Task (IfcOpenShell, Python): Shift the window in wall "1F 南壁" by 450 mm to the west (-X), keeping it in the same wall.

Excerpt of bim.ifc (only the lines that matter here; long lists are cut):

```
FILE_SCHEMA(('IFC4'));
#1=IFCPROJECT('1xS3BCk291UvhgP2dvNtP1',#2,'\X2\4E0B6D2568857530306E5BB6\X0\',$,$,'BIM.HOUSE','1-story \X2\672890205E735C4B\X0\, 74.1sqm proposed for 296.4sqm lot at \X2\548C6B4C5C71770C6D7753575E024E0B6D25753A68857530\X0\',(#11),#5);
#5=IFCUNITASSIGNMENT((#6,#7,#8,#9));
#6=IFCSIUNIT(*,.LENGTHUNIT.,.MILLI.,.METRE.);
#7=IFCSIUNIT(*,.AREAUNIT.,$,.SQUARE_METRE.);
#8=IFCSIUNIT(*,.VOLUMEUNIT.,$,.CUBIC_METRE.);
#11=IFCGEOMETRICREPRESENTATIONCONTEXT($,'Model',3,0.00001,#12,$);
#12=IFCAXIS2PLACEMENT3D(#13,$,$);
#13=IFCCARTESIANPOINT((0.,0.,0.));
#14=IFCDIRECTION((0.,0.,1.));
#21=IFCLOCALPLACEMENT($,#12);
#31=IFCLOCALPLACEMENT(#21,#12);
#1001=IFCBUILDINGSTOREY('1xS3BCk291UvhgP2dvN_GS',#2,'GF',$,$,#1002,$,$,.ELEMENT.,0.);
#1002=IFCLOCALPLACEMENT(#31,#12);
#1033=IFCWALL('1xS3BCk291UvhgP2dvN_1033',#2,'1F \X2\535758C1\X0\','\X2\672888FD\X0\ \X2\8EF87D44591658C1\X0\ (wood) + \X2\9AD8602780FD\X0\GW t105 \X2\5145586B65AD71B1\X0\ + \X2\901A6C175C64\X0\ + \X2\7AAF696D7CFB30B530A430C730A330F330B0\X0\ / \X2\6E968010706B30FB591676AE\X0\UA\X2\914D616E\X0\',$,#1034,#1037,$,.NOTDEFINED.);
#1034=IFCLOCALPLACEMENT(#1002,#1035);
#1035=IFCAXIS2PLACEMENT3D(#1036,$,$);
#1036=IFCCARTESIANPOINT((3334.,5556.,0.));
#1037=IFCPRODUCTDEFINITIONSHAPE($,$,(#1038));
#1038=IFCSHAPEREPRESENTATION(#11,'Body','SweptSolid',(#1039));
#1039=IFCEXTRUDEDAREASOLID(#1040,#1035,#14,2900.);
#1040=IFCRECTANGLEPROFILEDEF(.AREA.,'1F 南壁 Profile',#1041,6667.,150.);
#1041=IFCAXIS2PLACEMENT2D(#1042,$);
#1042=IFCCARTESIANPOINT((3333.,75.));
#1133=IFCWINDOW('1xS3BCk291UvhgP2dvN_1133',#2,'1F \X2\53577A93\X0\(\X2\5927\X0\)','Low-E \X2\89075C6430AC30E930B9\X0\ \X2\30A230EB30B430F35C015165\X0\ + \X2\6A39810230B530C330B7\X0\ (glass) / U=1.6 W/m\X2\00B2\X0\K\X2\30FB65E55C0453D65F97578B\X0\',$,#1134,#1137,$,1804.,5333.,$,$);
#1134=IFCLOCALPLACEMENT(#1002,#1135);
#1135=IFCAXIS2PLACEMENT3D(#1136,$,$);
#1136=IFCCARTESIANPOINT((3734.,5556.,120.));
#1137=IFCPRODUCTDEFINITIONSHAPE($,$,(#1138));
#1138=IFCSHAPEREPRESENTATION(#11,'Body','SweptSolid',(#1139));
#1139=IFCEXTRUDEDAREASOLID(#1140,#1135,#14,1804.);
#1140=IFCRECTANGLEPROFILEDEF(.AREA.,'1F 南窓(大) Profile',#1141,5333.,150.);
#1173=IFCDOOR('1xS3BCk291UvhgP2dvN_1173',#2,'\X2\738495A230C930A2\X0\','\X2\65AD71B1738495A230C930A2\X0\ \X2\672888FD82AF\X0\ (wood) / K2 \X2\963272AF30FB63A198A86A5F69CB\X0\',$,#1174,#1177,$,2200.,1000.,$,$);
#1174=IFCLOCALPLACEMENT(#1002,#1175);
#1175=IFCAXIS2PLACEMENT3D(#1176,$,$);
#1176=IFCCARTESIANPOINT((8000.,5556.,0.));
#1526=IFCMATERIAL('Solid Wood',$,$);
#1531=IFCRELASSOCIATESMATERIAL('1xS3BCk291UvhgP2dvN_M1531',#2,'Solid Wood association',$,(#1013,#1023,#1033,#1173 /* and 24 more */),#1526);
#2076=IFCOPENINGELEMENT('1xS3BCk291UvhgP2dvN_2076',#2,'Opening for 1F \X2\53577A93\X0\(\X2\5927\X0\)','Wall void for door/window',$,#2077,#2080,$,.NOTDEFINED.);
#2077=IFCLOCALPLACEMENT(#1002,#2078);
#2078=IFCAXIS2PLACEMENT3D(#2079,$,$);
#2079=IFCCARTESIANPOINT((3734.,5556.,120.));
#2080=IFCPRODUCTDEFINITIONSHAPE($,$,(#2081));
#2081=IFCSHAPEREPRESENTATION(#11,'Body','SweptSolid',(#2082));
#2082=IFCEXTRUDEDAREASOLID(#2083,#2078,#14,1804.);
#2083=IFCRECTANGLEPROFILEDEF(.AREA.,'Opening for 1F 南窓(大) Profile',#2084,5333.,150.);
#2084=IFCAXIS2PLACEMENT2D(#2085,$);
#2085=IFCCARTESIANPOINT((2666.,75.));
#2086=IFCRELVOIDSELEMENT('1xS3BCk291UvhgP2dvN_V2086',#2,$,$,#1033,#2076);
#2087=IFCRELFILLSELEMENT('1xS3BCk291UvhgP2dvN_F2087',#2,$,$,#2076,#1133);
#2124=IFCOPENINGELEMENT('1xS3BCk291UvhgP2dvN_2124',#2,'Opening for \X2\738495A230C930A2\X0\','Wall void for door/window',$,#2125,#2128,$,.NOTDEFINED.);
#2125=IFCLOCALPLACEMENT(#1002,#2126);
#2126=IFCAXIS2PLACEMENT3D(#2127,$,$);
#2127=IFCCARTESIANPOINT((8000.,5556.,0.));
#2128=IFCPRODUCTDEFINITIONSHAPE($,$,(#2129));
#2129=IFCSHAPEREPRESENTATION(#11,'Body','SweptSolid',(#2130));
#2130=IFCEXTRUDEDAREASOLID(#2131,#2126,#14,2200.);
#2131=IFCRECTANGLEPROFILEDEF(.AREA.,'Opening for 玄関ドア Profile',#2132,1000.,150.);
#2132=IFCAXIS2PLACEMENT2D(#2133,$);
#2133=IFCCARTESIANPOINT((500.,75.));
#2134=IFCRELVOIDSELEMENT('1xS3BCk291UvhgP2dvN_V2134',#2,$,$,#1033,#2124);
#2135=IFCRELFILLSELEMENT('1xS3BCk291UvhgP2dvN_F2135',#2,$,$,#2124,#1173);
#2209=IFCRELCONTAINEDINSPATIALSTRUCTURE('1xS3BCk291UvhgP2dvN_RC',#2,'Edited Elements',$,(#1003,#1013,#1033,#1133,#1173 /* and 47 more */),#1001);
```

```python
import ifcopenshell
import ifcopenshell.api.geometry
import ifcopenshell.util.placement
import ifcopenshell.util.unit

model = ifcopenshell.open("bim.ifc")
unit_scale = ifcopenshell.util.unit.calculate_unit_scale(model)

window = model.by_guid("1xS3BCk291UvhgP2dvN_1133")
opening = window.FillsVoids[0].RelatingOpeningElement
wall = opening.VoidsElements[0].RelatingBuildingElement

wall_matrix = ifcopenshell.util.placement.get_local_placement(wall.ObjectPlacement)
shift = wall_matrix[:3, 0] * -0.45 / unit_scale
before = ifcopenshell.util.placement.get_local_placement(window.ObjectPlacement)[:3, 3].copy()

# The window is not placed relative to its opening, so move both.
for product in (opening, window):
    matrix = ifcopenshell.util.placement.get_local_placement(product.ObjectPlacement)
    matrix[:3, 3] += shift
    ifcopenshell.api.geometry.edit_object_placement(model, product=product, matrix=matrix, is_si=False)

after = ifcopenshell.util.placement.get_local_placement(window.ObjectPlacement)[:3, 3]
print("window moved by", (after - before).round(3) + 0.0)

model.write("bim_edited.ifc")
```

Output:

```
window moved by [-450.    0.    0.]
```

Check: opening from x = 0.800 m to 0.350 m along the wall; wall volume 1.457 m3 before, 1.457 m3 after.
